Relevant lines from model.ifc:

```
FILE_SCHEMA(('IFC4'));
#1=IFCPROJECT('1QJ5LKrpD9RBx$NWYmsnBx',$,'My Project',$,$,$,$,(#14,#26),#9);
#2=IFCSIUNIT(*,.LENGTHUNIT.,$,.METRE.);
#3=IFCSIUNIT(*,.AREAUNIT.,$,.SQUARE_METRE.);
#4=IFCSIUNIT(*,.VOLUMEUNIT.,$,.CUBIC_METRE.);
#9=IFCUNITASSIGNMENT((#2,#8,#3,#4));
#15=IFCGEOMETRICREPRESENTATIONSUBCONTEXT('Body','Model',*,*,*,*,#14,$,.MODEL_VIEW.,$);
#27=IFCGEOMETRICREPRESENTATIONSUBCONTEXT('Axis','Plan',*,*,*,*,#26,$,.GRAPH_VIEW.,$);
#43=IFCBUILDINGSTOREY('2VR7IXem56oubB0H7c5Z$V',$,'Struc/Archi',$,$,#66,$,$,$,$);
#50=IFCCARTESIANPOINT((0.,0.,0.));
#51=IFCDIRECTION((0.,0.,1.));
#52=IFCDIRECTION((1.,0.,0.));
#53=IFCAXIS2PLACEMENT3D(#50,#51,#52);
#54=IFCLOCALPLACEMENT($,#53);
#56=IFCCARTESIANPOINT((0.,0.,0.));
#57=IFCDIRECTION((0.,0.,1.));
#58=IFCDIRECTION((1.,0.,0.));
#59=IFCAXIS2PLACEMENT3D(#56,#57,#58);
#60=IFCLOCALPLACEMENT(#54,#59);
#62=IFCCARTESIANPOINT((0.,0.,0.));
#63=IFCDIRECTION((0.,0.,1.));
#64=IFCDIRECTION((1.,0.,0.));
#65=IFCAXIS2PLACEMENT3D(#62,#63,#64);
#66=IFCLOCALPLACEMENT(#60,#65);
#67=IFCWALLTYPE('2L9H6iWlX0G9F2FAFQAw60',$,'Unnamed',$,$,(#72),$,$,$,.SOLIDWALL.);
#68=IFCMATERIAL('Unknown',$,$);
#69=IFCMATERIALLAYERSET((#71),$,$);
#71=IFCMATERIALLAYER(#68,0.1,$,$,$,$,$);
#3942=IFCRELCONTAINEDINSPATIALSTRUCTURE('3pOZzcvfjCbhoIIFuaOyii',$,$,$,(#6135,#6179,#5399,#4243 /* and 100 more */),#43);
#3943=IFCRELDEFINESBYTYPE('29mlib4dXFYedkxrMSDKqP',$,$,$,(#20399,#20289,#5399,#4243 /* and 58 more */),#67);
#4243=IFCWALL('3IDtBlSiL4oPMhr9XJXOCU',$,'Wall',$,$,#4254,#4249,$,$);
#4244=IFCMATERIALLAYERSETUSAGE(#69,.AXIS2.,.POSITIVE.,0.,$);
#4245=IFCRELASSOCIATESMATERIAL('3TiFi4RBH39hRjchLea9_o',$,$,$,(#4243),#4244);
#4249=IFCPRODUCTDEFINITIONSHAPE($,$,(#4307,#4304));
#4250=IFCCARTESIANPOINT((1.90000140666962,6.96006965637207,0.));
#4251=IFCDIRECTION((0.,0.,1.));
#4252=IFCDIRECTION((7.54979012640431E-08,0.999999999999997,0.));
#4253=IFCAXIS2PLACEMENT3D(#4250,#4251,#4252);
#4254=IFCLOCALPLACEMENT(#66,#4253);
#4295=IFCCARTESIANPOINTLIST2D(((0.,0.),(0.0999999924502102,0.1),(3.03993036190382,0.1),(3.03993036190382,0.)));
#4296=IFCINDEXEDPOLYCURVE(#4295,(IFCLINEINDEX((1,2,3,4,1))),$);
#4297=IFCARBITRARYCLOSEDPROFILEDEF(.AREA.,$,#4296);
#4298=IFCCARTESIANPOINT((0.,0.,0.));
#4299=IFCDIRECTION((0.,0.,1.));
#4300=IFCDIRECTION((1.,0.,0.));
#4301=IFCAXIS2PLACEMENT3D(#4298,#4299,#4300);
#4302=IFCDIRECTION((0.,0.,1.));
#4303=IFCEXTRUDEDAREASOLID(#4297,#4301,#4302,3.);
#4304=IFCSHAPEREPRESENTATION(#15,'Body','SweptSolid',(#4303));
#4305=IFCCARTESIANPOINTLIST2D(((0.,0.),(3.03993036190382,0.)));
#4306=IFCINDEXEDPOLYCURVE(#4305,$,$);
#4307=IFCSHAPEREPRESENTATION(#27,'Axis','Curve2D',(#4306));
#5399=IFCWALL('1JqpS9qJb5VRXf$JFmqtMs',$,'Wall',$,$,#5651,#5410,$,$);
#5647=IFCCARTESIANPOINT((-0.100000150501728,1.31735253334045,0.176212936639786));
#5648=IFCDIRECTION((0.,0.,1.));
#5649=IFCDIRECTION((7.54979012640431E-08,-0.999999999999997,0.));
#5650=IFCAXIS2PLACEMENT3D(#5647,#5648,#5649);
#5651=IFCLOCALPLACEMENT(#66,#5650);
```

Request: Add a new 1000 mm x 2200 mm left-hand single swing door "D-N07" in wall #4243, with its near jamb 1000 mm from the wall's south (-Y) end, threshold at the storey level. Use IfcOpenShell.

```python
import numpy as np
import ifcopenshell
import ifcopenshell.api.feature
import ifcopenshell.api.geometry
import ifcopenshell.api.root
import ifcopenshell.api.spatial
import ifcopenshell.geom
import ifcopenshell.util.element
import ifcopenshell.util.placement
import ifcopenshell.util.representation
import ifcopenshell.util.shape
import ifcopenshell.util.unit

model = ifcopenshell.open("model.ifc")
unit_scale = ifcopenshell.util.unit.calculate_unit_scale(model)
settings = ifcopenshell.geom.settings()


def volume(element):
    """Net volume in cubic metres, openings subtracted."""
    shape = ifcopenshell.geom.create_shape(settings, element)
    return ifcopenshell.util.shape.get_volume(shape.geometry)


wall = model.by_guid("3IDtBlSiL4oPMhr9XJXOCU")
storey = ifcopenshell.util.element.get_container(wall, ifc_class="IfcBuildingStorey")
context = ifcopenshell.util.representation.get_context(model, "Model", "Body", "MODEL_VIEW")
before = volume(wall)

width, height, from_end, sill = 1, 2.2, 1, 0.0  # metres

# The wall runs along its own X axis, and the end named is its -X end.
wall_shape = ifcopenshell.geom.create_shape(settings, wall)
x, y, z = ifcopenshell.util.shape.get_vertices(wall_shape.geometry).T
start = x.min() + from_end
face, thickness = float(y.min()), float(y.max() - y.min())
wall_matrix = ifcopenshell.util.placement.get_local_placement(wall.ObjectPlacement)
level = ifcopenshell.util.placement.get_local_placement(storey.ObjectPlacement)[2, 3]


def in_wall(x, y):
    """Placement at x, y metres in the wall's axes, at sill height."""
    matrix = wall_matrix.copy()
    matrix[:, 3] = wall_matrix @ np.array([x / unit_scale, y / unit_scale, 0.0, 1.0])
    matrix[2, 3] = level + sill / unit_scale
    return matrix


# Opening: a box that overshoots both wall faces by 50 mm.
opening = ifcopenshell.api.root.create_entity(model, ifc_class="IfcOpeningElement", predefined_type="OPENING")
box = ifcopenshell.api.geometry.add_wall_representation(
    model, context=context, length=width, height=height, thickness=thickness + 0.1
)
ifcopenshell.api.geometry.assign_representation(model, product=opening, representation=box)
ifcopenshell.api.geometry.edit_object_placement(model, product=opening, matrix=in_wall(start, face - 0.05), is_si=False)
ifcopenshell.api.feature.add_feature(model, feature=opening, element=wall)

door = ifcopenshell.api.root.create_entity(model, ifc_class="IfcDoor", name="D-N07", predefined_type="DOOR")
door.OverallWidth, door.OverallHeight = width / unit_scale, height / unit_scale
door.OperationType = "SINGLE_SWING_LEFT"
body = ifcopenshell.api.geometry.add_door_representation(
    model,
    context=context,
    overall_width=door.OverallWidth,
    overall_height=door.OverallHeight,
    operation_type="SINGLE_SWING_LEFT",
    lining_properties={"LiningDepth": thickness / unit_scale, "ThresholdDepth": thickness / unit_scale},
)
ifcopenshell.api.geometry.assign_representation(model, product=door, representation=body)
ifcopenshell.api.spatial.assign_container(model, products=[door], relating_structure=storey)
ifcopenshell.api.feature.add_filling(model, opening=opening, element=door)

# The lining spans the wall, so the door starts at the wall face.
ifcopenshell.api.geometry.edit_object_placement(model, product=door, matrix=in_wall(start, face), is_si=False)

after = volume(wall)

print(f"wall volume {before:.3f} -> {after:.3f} m3")

model.write("model_edited.ifc")
```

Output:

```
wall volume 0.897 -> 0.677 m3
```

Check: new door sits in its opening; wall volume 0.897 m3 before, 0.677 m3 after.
